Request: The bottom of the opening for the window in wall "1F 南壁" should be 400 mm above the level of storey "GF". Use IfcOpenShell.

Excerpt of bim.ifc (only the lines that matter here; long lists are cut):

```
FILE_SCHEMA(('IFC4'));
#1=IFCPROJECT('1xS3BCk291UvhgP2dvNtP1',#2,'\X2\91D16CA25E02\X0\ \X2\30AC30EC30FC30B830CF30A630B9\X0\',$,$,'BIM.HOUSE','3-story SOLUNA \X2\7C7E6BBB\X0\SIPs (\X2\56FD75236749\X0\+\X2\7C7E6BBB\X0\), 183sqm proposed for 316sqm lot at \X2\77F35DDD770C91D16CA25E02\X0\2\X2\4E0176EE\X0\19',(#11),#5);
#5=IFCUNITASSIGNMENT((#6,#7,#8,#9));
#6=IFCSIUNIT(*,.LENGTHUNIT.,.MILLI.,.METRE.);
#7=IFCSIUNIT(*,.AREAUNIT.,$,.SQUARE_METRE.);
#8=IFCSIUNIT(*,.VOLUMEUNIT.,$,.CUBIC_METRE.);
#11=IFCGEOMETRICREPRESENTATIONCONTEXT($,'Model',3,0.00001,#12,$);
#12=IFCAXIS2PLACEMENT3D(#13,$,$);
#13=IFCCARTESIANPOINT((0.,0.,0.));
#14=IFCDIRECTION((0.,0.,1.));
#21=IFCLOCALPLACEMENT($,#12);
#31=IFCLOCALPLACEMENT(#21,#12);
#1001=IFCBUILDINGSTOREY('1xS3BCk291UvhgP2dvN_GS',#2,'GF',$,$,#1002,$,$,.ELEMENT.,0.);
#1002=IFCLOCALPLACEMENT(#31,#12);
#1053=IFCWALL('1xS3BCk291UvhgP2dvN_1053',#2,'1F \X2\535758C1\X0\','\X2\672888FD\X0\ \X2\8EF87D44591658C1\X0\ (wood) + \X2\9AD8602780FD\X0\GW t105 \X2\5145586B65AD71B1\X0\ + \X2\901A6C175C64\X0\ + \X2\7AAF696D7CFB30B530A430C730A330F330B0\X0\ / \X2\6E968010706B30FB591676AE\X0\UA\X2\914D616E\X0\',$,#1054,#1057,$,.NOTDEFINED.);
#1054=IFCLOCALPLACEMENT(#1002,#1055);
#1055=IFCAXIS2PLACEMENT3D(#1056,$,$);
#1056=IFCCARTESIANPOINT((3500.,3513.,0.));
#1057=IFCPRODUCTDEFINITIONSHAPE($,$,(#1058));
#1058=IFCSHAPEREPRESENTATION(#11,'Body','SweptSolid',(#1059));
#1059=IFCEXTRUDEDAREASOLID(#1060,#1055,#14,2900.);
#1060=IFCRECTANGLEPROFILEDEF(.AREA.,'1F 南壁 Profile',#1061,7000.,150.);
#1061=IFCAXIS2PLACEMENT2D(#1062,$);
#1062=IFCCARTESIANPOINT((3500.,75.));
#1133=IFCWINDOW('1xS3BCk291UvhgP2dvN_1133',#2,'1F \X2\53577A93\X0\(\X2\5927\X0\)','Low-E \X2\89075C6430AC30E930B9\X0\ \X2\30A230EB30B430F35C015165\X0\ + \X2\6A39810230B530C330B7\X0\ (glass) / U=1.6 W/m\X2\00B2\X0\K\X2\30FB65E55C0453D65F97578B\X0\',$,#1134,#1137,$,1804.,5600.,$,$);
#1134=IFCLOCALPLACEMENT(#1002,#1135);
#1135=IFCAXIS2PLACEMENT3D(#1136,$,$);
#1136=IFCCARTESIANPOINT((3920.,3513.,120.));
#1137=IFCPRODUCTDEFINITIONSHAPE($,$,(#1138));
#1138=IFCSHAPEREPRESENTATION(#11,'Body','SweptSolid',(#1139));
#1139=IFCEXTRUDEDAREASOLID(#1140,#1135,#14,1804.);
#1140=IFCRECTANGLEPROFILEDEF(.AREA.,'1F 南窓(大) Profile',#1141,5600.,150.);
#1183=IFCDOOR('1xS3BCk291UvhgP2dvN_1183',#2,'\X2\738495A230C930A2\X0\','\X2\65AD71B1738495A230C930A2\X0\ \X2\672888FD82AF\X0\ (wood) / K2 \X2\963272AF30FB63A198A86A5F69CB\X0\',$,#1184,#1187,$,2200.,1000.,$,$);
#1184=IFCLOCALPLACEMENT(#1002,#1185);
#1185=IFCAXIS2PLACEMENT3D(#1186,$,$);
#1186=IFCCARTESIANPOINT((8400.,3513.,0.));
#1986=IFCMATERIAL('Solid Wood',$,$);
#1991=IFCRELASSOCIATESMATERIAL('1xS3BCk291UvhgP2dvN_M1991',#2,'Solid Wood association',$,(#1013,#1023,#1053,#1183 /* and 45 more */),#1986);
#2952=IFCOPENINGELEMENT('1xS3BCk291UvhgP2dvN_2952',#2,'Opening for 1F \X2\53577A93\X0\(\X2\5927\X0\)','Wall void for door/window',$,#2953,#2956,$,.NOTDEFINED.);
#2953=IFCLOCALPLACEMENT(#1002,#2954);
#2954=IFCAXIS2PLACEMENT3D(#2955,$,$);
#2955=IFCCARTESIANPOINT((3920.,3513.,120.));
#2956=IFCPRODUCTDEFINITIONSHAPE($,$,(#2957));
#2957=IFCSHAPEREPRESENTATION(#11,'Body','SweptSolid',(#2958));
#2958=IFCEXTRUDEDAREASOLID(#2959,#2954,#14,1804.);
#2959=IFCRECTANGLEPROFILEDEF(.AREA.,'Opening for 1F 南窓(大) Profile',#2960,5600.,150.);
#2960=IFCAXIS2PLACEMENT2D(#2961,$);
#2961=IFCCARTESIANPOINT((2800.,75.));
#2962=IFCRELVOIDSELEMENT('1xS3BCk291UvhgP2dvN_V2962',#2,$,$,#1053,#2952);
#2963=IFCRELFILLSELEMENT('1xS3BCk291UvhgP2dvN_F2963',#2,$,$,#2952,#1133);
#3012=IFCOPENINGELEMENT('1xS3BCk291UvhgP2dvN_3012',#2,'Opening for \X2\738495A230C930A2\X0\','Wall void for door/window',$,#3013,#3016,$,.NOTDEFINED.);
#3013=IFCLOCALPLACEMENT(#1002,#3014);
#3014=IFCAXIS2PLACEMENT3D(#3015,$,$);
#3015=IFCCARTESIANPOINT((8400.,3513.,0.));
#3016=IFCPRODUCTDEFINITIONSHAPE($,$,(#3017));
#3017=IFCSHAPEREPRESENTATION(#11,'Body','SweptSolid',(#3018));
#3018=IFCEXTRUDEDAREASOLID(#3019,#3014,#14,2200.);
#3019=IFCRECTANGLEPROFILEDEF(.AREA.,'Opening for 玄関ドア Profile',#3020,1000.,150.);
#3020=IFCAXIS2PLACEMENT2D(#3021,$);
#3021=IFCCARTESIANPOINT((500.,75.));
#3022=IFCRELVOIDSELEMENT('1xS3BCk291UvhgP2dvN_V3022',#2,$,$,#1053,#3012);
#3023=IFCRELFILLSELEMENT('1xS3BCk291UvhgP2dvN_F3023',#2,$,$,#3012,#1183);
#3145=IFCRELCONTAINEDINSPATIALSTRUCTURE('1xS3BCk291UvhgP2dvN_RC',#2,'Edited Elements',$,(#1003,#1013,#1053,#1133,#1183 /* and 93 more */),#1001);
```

```python
import numpy as np
import ifcopenshell
import ifcopenshell.api.geometry
import ifcopenshell.geom
import ifcopenshell.util.element
import ifcopenshell.util.placement
import ifcopenshell.util.shape
import ifcopenshell.util.unit

model = ifcopenshell.open("bim.ifc")
unit_scale = ifcopenshell.util.unit.calculate_unit_scale(model)

window = model.by_id(1133)
opening = window.FillsVoids[0].RelatingOpeningElement
storey = ifcopenshell.util.element.get_container(window, ifc_class="IfcBuildingStorey")
level = ifcopenshell.util.placement.get_local_placement(storey.ObjectPlacement)[2, 3]

# The opening's origin need not be at the sill, so measure its lowest point.
shape = ifcopenshell.geom.create_shape(ifcopenshell.geom.settings(), opening)
bottom = ifcopenshell.util.shape.get_shape_bottom_elevation(shape, shape.geometry) / unit_scale
dz = level + 0.4 / unit_scale - bottom

shift = np.array([0.0, 0.0, dz])
# The window is not placed relative to its opening, so move both.
for product in (opening, window):
    matrix = ifcopenshell.util.placement.get_local_placement(product.ObjectPlacement)
    matrix[:3, 3] += shift
    ifcopenshell.api.geometry.edit_object_placement(model, product=product, matrix=matrix, is_si=False)

print(f"moved by {dz * unit_scale:+.3f} m")

model.write("bim_v2.ifc")
```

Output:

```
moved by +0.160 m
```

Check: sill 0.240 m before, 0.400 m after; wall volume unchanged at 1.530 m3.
